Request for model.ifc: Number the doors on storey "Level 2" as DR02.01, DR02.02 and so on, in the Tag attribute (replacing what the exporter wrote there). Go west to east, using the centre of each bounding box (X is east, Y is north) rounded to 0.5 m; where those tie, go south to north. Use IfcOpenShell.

First a look at what the model holds.

```python
import ifcopenshell
import ifcopenshell.util.element
import ifcopenshell.util.placement

model = ifcopenshell.open("model.ifc")
print(model.schema)
storey = next(s for s in model.by_type("IfcBuildingStorey") if s.Name == "Level 2")
doors = [e for e in ifcopenshell.util.element.get_decomposition(storey) if e.is_a("IfcDoor")]
for e in sorted(doors, key=lambda e: e.id()):
    origin = ifcopenshell.util.placement.get_local_placement(e.ObjectPlacement)[:3, 3]
    print(e.id(), e.Tag, e.Name, origin.round(2) + 0.0, sep=" | ")
```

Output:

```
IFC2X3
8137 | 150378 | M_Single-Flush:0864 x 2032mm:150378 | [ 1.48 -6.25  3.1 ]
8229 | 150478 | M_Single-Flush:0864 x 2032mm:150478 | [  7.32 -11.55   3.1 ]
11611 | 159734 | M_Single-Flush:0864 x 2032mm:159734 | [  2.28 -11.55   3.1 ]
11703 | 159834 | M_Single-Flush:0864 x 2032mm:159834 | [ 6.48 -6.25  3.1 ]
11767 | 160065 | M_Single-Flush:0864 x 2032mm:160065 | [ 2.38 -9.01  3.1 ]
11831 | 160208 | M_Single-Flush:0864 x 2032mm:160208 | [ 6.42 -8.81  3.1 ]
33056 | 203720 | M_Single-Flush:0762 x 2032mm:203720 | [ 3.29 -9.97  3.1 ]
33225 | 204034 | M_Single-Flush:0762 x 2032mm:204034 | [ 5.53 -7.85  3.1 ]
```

```python
import ifcopenshell
import ifcopenshell.geom
import ifcopenshell.util.element
import ifcopenshell.util.shape

model = ifcopenshell.open("model.ifc")
settings = ifcopenshell.geom.settings()
settings.set("use-world-coords", True)


def centre(element):
    shape = ifcopenshell.geom.create_shape(settings, element)
    return ifcopenshell.util.shape.get_bbox_centroid(shape.geometry)


storey = next(s for s in model.by_type("IfcBuildingStorey") if s.Name == "Level 2")
doors = [e for e in ifcopenshell.util.element.get_decomposition(storey) if e.is_a("IfcDoor")]

# Insertion points can sit at a corner or the storey origin, so sort by the geometry (in metres).
centres = {e: centre(e) for e in doors}
doors.sort(key=lambda e: (round(centres[e][0] / 0.5), centres[e][1]))

for i, e in enumerate(doors, start=1):
    number = f"DR02.{i:02d}"
    e.Tag = number
    print(e.id(), number)

model.write("model_rev.ifc")
```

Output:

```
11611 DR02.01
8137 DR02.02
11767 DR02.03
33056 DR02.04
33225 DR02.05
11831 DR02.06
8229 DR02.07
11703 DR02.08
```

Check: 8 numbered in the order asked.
